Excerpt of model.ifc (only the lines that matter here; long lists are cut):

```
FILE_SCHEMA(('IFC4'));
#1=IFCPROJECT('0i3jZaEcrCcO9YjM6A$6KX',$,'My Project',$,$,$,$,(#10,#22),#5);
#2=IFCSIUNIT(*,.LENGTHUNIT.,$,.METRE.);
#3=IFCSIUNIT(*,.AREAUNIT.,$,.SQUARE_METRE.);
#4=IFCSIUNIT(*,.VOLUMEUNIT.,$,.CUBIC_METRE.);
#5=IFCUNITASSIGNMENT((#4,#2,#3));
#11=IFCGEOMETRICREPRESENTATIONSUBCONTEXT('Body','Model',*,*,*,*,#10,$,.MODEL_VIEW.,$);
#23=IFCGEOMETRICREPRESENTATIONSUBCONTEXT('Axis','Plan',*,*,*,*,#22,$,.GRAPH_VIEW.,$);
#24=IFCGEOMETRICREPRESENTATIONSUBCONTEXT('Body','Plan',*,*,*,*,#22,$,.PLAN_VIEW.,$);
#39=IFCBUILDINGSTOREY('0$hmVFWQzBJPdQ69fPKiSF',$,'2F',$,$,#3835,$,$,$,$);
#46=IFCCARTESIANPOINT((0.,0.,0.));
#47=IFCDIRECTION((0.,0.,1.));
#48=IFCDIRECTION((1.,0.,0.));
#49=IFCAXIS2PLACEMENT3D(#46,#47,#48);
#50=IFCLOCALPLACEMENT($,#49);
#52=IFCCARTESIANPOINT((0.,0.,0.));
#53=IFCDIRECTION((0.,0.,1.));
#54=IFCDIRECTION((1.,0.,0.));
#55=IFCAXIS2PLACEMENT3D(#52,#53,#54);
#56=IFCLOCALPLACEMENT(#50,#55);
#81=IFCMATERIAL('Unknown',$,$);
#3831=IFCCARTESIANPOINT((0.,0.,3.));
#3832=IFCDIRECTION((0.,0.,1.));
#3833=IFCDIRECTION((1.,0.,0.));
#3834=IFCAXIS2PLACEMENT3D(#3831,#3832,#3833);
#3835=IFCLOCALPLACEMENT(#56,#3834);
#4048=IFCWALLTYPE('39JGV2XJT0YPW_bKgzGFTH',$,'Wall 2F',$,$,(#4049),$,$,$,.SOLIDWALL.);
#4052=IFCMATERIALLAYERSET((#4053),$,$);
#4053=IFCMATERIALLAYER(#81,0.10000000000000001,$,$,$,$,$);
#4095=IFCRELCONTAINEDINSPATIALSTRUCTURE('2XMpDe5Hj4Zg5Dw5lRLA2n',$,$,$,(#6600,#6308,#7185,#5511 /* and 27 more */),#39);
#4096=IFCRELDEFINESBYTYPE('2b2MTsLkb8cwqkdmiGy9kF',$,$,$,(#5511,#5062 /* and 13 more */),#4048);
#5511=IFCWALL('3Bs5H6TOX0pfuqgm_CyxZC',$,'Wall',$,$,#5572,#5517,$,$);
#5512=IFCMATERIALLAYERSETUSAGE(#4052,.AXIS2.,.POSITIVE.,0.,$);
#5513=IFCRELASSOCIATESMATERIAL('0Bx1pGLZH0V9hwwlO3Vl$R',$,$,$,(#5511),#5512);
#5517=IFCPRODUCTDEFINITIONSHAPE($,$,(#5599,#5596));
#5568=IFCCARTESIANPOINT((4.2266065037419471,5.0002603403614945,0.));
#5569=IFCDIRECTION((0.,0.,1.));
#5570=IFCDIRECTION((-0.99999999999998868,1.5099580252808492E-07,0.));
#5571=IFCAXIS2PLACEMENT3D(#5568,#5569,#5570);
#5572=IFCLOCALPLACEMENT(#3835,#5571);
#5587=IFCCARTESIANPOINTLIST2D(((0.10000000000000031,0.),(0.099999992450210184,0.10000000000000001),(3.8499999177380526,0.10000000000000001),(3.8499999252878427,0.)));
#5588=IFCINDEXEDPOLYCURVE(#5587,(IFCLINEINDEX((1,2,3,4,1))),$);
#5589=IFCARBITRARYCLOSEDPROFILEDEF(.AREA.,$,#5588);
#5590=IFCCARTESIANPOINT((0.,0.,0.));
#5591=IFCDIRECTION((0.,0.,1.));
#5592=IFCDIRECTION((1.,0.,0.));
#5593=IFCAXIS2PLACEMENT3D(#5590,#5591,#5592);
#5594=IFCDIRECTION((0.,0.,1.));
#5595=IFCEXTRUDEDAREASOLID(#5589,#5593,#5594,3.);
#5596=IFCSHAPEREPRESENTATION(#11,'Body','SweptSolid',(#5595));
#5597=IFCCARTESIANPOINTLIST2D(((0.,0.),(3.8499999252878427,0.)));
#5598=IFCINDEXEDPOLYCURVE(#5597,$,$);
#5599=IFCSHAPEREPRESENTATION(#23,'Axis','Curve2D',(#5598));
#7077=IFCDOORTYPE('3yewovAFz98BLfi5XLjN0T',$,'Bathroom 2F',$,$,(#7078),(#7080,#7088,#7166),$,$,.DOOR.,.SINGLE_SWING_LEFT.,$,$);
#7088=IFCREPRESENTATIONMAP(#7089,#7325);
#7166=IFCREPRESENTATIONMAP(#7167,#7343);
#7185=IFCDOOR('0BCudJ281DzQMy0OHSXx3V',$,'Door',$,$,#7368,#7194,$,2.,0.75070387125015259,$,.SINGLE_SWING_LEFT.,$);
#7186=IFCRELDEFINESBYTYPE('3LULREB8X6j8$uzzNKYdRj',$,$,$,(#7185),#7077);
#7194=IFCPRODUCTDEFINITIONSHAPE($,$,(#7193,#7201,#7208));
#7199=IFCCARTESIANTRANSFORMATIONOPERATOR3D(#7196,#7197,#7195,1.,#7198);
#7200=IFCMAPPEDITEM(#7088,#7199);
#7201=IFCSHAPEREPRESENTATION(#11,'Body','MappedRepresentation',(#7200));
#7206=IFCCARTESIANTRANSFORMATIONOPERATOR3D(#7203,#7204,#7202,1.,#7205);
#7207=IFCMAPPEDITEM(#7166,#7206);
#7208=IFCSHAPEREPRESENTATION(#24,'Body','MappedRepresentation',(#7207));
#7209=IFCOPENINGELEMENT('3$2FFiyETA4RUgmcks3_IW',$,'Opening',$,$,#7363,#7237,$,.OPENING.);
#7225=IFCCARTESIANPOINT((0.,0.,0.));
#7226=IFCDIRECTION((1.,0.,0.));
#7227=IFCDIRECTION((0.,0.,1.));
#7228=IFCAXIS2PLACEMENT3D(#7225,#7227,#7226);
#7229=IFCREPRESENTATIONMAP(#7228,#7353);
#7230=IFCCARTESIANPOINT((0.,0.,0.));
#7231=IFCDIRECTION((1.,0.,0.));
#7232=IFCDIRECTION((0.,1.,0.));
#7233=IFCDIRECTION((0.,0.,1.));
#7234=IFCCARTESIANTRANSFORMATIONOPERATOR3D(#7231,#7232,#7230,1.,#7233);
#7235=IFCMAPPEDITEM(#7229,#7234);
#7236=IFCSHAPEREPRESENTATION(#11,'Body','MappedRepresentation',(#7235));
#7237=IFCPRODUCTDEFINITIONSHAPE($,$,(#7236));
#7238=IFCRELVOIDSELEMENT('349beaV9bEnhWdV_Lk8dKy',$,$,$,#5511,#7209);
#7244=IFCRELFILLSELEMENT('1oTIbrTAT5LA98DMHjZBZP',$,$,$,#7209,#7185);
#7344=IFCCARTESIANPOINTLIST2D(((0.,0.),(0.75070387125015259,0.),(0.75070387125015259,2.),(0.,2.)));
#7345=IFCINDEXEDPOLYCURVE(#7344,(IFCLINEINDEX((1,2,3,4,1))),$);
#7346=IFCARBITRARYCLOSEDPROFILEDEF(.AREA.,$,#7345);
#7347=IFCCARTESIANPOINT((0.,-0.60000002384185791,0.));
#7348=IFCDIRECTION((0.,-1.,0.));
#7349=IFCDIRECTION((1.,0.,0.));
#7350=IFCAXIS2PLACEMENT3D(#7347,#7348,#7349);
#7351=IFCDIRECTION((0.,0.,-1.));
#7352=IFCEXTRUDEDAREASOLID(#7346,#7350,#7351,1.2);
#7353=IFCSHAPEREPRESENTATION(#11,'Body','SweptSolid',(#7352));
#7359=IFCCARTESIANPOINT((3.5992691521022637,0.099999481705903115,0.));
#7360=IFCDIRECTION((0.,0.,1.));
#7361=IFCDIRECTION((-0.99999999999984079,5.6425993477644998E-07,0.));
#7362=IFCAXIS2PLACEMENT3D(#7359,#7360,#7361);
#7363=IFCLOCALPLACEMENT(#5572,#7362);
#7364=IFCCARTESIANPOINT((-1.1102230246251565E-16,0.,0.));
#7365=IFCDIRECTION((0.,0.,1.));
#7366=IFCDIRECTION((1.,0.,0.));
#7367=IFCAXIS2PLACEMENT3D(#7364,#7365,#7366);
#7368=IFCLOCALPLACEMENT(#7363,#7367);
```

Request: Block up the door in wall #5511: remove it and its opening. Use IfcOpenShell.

```python
import ifcopenshell
import ifcopenshell.api.feature
import ifcopenshell.api.root
import ifcopenshell.geom
import ifcopenshell.util.shape

model = ifcopenshell.open("model.ifc")
settings = ifcopenshell.geom.settings()


def volume(element):
    """Net volume in cubic metres, openings subtracted."""
    shape = ifcopenshell.geom.create_shape(settings, element)
    return ifcopenshell.util.shape.get_volume(shape.geometry)


door = model.by_guid("0BCudJ281DzQMy0OHSXx3V")
opening = door.FillsVoids[0].RelatingOpeningElement
wall = opening.VoidsElements[0].RelatingBuildingElement
before = volume(wall)

ifcopenshell.api.root.remove_product(model, product=door)
ifcopenshell.api.feature.remove_feature(model, feature=opening)

after = volume(wall)

print(f"wall volume {before:.3f} -> {after:.3f} m3")

model.write("model_edited.ifc")
```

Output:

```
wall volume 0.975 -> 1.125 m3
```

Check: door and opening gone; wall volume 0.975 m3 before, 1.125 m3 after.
